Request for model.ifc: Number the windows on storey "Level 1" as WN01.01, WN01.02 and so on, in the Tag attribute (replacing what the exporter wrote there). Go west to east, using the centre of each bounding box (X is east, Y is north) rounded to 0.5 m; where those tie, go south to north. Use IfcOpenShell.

First a look at what the model holds.

```python
import ifcopenshell
import ifcopenshell.util.element
import ifcopenshell.util.placement

model = ifcopenshell.open("model.ifc")
print(model.schema)
storey = next(s for s in model.by_type("IfcBuildingStorey") if s.Name == "Level 1")
windows = [e for e in ifcopenshell.util.element.get_decomposition(storey) if e.is_a("IfcWindow")]
for e in sorted(windows, key=lambda e: e.id()):
    origin = ifcopenshell.util.placement.get_local_placement(e.ObjectPlacement)[:3, 3]
    print(e.id(), e.Tag, e.Name, origin.round(2) + 0.0, sep=" | ")
```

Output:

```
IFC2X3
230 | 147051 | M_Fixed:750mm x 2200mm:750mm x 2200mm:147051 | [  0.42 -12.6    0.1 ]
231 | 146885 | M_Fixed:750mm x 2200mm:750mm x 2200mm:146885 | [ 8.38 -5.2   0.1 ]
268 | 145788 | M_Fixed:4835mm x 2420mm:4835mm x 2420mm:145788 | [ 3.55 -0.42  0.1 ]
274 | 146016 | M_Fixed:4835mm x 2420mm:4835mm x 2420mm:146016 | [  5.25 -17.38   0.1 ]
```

```python
import ifcopenshell
import ifcopenshell.geom
import ifcopenshell.util.element
import ifcopenshell.util.shape

model = ifcopenshell.open("model.ifc")
settings = ifcopenshell.geom.settings()
settings.set("use-world-coords", True)


def centre(element):
    shape = ifcopenshell.geom.create_shape(settings, element)
    return ifcopenshell.util.shape.get_bbox_centroid(shape.geometry)


storey = next(s for s in model.by_type("IfcBuildingStorey") if s.Name == "Level 1")
windows = [e for e in ifcopenshell.util.element.get_decomposition(storey) if e.is_a("IfcWindow")]

# Insertion points can sit at a corner or the storey origin, so sort by the geometry (in metres).
centres = {e: centre(e) for e in windows}
windows.sort(key=lambda e: (round(centres[e][0] / 0.5), centres[e][1]))

for i, e in enumerate(windows, start=1):
    number = f"WN01.{i:02d}"
    e.Tag = number
    print(e.id(), number)

model.write("model_rev.ifc")
```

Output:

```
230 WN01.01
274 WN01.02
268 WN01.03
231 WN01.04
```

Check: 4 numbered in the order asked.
